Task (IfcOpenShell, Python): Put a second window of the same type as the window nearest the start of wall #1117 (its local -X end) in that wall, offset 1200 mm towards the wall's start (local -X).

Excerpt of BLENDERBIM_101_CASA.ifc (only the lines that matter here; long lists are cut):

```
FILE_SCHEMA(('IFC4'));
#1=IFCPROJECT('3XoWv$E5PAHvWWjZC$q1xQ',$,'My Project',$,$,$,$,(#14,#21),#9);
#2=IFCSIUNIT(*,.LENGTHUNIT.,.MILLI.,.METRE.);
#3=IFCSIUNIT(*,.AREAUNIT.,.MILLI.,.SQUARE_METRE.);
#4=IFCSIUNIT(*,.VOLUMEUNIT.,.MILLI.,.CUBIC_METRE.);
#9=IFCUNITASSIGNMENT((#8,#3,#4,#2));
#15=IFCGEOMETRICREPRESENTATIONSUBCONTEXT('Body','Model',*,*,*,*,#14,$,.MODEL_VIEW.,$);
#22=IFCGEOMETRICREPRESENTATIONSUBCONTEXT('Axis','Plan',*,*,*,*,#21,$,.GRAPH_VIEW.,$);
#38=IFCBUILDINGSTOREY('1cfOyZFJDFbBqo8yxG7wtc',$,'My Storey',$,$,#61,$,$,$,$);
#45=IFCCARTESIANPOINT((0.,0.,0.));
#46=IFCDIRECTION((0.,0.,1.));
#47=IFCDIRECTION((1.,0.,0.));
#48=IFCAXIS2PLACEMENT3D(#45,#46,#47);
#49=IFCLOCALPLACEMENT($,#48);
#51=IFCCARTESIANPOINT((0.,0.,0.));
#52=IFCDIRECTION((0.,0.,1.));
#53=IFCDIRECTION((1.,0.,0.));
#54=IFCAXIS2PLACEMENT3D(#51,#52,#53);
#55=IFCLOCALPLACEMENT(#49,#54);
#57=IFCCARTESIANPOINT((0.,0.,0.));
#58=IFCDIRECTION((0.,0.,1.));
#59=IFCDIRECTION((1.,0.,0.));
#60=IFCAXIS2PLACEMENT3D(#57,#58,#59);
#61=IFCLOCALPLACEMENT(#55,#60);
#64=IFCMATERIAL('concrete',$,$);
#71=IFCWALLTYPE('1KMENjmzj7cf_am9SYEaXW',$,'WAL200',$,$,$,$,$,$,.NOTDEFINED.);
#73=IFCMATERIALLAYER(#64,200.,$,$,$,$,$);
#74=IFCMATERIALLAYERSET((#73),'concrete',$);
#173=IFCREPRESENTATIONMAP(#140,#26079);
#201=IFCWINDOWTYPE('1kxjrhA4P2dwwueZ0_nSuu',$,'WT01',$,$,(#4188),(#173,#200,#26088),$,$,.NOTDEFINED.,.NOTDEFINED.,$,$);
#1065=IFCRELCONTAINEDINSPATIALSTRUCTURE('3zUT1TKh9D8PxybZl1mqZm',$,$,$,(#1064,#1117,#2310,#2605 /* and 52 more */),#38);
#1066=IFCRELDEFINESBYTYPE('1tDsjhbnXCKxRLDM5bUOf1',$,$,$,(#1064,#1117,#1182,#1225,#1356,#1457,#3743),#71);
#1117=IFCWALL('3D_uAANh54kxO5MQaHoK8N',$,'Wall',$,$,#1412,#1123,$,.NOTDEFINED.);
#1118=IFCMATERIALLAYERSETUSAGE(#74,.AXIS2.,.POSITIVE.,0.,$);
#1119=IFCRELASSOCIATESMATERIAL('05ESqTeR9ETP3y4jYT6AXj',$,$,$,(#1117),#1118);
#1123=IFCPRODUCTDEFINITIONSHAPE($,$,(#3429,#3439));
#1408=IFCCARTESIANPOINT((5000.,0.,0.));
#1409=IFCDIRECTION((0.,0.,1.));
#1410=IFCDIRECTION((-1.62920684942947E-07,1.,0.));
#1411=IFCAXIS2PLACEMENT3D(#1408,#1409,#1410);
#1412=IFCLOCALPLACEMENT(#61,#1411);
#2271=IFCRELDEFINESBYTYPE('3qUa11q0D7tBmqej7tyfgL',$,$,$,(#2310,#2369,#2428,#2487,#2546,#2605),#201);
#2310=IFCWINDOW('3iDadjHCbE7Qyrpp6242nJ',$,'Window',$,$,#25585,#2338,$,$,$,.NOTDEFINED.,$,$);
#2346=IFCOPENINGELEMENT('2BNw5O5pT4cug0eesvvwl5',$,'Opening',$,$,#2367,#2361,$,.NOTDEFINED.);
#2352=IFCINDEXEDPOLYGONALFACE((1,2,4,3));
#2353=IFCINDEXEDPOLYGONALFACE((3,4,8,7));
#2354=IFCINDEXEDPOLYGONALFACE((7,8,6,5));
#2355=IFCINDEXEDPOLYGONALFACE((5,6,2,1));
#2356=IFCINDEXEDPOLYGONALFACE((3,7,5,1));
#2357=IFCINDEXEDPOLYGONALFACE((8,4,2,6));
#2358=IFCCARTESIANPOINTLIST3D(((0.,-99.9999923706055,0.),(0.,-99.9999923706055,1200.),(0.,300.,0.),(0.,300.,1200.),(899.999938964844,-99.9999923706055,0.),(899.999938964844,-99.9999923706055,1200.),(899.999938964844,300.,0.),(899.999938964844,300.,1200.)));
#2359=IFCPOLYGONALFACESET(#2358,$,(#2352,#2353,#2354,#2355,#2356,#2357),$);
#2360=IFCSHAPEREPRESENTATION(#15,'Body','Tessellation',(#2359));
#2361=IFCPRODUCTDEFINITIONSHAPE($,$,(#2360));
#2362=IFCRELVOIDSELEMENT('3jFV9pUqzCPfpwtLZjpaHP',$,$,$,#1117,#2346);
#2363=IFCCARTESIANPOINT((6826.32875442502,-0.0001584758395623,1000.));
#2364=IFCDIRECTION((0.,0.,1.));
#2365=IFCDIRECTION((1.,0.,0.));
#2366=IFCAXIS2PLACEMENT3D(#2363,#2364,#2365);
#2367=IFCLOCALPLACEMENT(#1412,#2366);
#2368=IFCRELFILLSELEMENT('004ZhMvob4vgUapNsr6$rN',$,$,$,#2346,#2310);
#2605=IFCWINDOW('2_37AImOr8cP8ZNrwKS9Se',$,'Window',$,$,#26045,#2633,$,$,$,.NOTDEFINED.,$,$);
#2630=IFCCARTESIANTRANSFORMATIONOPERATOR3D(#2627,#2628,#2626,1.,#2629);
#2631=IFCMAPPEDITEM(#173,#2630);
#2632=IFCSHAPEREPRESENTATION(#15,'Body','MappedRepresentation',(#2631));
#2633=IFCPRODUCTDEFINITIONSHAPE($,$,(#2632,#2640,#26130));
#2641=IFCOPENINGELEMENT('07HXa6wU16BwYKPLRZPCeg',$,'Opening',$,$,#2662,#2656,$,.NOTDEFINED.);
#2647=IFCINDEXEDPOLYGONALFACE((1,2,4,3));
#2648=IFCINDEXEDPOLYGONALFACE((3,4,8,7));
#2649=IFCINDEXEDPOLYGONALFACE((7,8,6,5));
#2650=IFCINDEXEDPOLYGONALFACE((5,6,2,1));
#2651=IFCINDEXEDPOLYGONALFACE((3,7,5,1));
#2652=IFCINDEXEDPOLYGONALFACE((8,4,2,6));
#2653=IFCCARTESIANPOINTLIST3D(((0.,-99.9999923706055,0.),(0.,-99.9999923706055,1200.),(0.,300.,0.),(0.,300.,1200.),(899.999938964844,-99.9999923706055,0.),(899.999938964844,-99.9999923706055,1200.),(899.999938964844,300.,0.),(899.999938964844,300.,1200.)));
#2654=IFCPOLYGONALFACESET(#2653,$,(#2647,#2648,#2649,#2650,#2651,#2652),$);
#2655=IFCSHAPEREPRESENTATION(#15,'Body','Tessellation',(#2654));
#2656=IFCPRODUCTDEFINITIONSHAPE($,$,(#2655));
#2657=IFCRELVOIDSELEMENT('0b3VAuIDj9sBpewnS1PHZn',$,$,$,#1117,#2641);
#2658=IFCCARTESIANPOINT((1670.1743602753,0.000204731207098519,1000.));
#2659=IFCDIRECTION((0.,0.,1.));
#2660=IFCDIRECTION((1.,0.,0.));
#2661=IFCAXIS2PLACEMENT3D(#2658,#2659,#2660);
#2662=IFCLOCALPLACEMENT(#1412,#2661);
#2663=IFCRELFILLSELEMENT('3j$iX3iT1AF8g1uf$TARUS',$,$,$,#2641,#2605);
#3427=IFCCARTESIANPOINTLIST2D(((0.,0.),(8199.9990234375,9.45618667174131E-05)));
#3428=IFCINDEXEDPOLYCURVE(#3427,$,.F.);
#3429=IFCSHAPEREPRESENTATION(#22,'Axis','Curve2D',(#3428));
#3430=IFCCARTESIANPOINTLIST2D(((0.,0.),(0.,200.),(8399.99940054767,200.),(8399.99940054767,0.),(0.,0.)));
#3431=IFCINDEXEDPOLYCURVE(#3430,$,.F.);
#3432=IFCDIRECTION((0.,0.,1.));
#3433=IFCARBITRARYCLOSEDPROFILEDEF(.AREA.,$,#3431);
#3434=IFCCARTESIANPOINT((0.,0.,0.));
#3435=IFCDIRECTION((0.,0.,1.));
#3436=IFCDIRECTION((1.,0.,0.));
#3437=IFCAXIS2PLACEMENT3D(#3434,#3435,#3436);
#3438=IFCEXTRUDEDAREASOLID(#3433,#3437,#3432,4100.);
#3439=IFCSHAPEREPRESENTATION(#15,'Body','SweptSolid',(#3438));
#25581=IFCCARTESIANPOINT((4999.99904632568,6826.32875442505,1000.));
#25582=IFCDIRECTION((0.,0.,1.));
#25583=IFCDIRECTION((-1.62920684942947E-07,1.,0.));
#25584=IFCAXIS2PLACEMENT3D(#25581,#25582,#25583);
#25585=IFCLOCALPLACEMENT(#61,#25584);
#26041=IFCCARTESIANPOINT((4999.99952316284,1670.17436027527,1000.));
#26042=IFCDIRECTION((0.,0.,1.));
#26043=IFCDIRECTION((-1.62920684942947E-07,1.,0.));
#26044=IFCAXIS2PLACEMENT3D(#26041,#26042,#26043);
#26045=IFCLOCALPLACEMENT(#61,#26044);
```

```python
import ifcopenshell
import ifcopenshell.api.feature
import ifcopenshell.api.geometry
import ifcopenshell.api.root
import ifcopenshell.geom
import ifcopenshell.util.element
import ifcopenshell.util.placement
import ifcopenshell.util.shape

model = ifcopenshell.open("BLENDERBIM_101_CASA.ifc")
settings = ifcopenshell.geom.settings()


def volume(element):
    """Net volume in cubic metres, openings subtracted."""
    shape = ifcopenshell.geom.create_shape(settings, element)
    return ifcopenshell.util.shape.get_volume(shape.geometry)


window = model.by_guid("2_37AImOr8cP8ZNrwKS9Se")
opening = window.FillsVoids[0].RelatingOpeningElement
wall = opening.VoidsElements[0].RelatingBuildingElement
before = volume(wall)
shift = ifcopenshell.util.placement.get_local_placement(wall.ObjectPlacement)[:3, 0] * -1200.0

# copy_class copies the void relationship, type, container and properties, but no geometry.
new_opening = ifcopenshell.api.root.copy_class(model, product=opening)
new_opening.Representation = ifcopenshell.util.element.copy_deep(
    model, opening.Representation, exclude=["IfcGeometricRepresentationContext", "IfcRepresentationMap"]
)
new_window = ifcopenshell.api.root.copy_class(model, product=window)
new_window.Representation = ifcopenshell.util.element.copy_deep(
    model, window.Representation, exclude=["IfcGeometricRepresentationContext", "IfcRepresentationMap"]
)
ifcopenshell.api.feature.add_filling(model, opening=new_opening, element=new_window)

for old, new in ((opening, new_opening), (window, new_window)):
    matrix = ifcopenshell.util.placement.get_local_placement(old.ObjectPlacement)
    matrix[:3, 3] += shift
    ifcopenshell.api.geometry.edit_object_placement(model, product=new, matrix=matrix, is_si=False)

after = volume(wall)

print(f"wall volume {before:.3f} -> {after:.3f} m3")

model.write("BLENDERBIM_101_CASA_rev.ifc")
```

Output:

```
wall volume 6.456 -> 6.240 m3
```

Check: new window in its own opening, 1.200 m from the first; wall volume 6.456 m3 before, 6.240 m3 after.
